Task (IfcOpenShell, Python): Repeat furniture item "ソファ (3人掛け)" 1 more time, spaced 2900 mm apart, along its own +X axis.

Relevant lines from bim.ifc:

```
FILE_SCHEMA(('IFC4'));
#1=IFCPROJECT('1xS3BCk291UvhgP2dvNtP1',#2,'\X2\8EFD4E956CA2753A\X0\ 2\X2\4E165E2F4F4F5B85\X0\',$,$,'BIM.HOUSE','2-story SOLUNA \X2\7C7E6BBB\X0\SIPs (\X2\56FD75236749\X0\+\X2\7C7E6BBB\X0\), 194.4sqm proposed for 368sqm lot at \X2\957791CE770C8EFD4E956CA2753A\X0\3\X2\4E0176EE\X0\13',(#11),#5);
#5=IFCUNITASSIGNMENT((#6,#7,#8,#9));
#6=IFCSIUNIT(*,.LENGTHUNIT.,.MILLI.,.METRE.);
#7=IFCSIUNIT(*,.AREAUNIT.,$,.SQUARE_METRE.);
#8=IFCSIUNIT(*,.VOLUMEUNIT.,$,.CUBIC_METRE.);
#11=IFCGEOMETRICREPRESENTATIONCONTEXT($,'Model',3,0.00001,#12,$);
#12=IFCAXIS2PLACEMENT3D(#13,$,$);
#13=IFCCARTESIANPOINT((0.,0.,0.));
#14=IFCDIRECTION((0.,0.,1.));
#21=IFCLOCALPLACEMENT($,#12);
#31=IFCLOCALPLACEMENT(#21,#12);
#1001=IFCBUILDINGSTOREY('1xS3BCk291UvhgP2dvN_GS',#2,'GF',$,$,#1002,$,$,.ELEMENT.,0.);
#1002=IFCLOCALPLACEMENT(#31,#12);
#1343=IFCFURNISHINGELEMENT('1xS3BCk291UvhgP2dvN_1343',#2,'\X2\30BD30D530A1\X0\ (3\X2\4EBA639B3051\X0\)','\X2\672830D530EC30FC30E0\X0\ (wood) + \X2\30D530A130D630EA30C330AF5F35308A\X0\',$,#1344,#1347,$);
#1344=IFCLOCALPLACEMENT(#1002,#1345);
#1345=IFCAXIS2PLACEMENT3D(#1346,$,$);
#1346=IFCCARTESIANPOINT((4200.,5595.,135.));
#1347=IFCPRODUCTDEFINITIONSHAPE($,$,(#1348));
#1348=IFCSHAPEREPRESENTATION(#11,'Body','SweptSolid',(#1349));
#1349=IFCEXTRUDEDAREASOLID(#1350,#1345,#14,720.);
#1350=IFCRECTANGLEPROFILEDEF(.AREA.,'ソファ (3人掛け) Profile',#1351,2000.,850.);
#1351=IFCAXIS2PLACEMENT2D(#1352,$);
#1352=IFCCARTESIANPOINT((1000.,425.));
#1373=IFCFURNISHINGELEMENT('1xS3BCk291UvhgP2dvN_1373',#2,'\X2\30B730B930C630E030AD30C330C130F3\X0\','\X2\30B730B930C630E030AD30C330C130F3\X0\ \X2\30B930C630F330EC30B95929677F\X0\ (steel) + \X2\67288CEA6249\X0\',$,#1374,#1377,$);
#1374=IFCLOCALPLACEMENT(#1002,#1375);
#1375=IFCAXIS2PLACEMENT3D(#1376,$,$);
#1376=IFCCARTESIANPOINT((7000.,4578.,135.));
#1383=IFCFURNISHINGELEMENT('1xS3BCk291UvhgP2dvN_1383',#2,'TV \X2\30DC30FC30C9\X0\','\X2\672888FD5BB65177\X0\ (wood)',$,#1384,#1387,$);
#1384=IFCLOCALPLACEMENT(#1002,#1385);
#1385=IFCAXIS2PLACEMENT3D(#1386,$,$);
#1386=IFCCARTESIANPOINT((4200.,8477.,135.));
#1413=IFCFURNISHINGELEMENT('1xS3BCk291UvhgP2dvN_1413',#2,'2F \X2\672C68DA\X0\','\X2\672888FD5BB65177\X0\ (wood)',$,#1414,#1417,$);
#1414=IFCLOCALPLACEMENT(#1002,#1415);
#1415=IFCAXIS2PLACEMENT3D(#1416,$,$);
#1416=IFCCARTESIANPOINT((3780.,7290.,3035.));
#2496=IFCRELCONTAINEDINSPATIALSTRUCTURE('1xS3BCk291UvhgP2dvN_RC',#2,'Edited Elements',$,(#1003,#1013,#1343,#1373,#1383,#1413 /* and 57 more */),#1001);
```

```python
import ifcopenshell
import ifcopenshell.api.geometry
import ifcopenshell.api.root
import ifcopenshell.util.element
import ifcopenshell.util.placement
import ifcopenshell.util.unit

model = ifcopenshell.open("bim.ifc")
unit_scale = ifcopenshell.util.unit.calculate_unit_scale(model)


def reuse_history(source, copy):
    """copy_class also copies each property set's owner history, people and application; keep the originals."""
    for rel in copy.IsDefinedBy:
        if rel.is_a("IfcRelDefinesByProperties") and (history := rel.RelatingPropertyDefinition.OwnerHistory):
            rel.RelatingPropertyDefinition.OwnerHistory = source.OwnerHistory
            ifcopenshell.util.element.remove_deep2(model, history)


source = model.by_guid("1xS3BCk291UvhgP2dvN_1343")
base = ifcopenshell.util.placement.get_local_placement(source.ObjectPlacement)
step = base[:3, 0] * 2.9 / unit_scale

for i in range(1, 2):
    copy = ifcopenshell.api.root.copy_class(model, product=source)
    copy.Representation = ifcopenshell.util.element.copy_deep(
        model, source.Representation, exclude=["IfcGeometricRepresentationContext", "IfcRepresentationMap"]
    )
    reuse_history(source, copy)
    matrix = base.copy()
    matrix[:3, 3] += i * step
    print("added at", matrix[:3, 3].round(3) + 0.0)
    ifcopenshell.api.geometry.edit_object_placement(model, product=copy, matrix=matrix, is_si=False)

model.write("bim_rev.ifc")
```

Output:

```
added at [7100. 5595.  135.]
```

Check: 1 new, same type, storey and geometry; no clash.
